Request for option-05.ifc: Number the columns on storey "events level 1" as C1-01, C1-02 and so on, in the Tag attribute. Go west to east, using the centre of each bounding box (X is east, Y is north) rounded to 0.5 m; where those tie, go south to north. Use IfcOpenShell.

First a look at what the model holds.

```python
import ifcopenshell
import ifcopenshell.util.element
import ifcopenshell.util.placement

model = ifcopenshell.open("option-05.ifc")
print(model.schema)
storey = next(s for s in model.by_type("IfcBuildingStorey") if s.Name == "events level 1")
columns = [e for e in ifcopenshell.util.element.get_decomposition(storey) if e.is_a("IfcColumn")]
for e in sorted(columns, key=lambda e: e.id()):
    origin = ifcopenshell.util.placement.get_local_placement(e.ObjectPlacement)[:3, 3]
    print(e.id(), e.Tag, e.Name, origin.round(2) + 0.0, sep=" | ")
```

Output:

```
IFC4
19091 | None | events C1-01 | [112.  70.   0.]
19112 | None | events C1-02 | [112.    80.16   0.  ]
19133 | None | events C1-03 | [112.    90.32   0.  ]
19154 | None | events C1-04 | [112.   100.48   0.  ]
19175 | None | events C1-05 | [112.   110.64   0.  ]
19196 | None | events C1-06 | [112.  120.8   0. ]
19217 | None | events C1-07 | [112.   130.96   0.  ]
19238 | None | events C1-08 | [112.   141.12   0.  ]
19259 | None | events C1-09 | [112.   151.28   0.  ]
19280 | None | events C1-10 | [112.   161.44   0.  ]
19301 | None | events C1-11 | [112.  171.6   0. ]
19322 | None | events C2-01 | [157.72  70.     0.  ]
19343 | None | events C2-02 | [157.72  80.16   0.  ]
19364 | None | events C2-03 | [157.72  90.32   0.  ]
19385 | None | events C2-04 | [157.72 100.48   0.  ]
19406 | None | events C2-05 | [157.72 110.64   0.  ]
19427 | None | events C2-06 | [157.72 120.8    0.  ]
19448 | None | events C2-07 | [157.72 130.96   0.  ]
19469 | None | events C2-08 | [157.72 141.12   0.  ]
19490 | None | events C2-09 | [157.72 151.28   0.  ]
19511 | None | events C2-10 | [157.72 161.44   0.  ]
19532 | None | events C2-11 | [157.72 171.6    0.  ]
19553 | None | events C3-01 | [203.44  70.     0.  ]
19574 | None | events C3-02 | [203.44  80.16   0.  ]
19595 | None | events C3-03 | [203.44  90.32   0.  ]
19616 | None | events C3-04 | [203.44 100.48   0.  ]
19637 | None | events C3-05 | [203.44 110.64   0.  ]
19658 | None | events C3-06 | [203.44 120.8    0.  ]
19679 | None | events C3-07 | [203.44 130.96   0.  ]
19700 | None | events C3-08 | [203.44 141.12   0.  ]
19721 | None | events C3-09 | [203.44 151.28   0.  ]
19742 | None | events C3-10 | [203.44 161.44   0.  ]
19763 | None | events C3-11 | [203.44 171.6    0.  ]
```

```python
import ifcopenshell
import ifcopenshell.geom
import ifcopenshell.util.element
import ifcopenshell.util.shape

model = ifcopenshell.open("option-05.ifc")
settings = ifcopenshell.geom.settings()
settings.set("use-world-coords", True)


def centre(element):
    shape = ifcopenshell.geom.create_shape(settings, element)
    return ifcopenshell.util.shape.get_bbox_centroid(shape.geometry)


storey = next(s for s in model.by_type("IfcBuildingStorey") if s.Name == "events level 1")
columns = [e for e in ifcopenshell.util.element.get_decomposition(storey) if e.is_a("IfcColumn")]

# Insertion points can sit at a corner or the storey origin, so sort by the geometry (in metres).
centres = {e: centre(e) for e in columns}
columns.sort(key=lambda e: (round(centres[e][0] / 0.5), centres[e][1]))

for i, e in enumerate(columns, start=1):
    number = f"C1-{i:02d}"
    e.Tag = number
    print(e.id(), number)

model.write("option-05_updated.ifc")
```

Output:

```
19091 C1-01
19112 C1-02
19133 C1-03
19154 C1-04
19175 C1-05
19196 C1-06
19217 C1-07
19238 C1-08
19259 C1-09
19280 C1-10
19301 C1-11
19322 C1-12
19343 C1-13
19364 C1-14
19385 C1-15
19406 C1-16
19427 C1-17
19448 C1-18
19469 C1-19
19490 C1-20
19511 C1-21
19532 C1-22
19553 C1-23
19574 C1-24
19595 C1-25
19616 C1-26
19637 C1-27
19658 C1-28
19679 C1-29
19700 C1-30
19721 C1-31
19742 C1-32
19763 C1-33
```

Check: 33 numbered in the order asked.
